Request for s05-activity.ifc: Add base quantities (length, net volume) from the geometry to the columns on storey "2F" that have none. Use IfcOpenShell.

First a look at what the model holds.

```python
import ifcopenshell
import ifcopenshell.util.element
import ifcopenshell.util.unit

model = ifcopenshell.open("s05-activity.ifc")
print(model.schema)
for unit_type in ("LENGTHUNIT", "AREAUNIT", "VOLUMEUNIT"):
    print(unit_type, ifcopenshell.util.unit.calculate_unit_scale(model, unit_type))
storey = next(s for s in model.by_type("IfcBuildingStorey") if s.Name == "2F")
columns = [e for e in ifcopenshell.util.element.get_decomposition(storey) if e.is_a("IfcColumn")]
for e in sorted(columns, key=lambda e: e.id()):
    print(e.id(), e.is_a(), e.Name, list(ifcopenshell.util.element.get_psets(e, qtos_only=True)), sep=" | ")
```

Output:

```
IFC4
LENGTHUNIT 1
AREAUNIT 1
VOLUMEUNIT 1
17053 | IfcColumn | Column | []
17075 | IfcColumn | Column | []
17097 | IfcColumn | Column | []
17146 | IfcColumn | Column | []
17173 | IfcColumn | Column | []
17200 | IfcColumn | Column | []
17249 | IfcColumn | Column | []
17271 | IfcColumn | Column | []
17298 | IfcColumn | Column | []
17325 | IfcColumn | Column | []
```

```python
import ifcopenshell
import ifcopenshell.api.pset
import ifcopenshell.geom
import ifcopenshell.util.element
import ifcopenshell.util.shape
import ifcopenshell.util.unit

model = ifcopenshell.open("s05-activity.ifc")
unit_scale = ifcopenshell.util.unit.calculate_unit_scale(model)
volume_scale = ifcopenshell.util.unit.calculate_unit_scale(model, "VOLUMEUNIT")
settings = ifcopenshell.geom.settings()

storey = next(s for s in model.by_type("IfcBuildingStorey") if s.Name == "2F")
columns = [e for e in ifcopenshell.util.element.get_decomposition(storey) if e.is_a("IfcColumn")]

for e in sorted(columns, key=lambda e: e.id()):
    if ifcopenshell.util.element.get_psets(e, qtos_only=True, should_inherit=False):
        continue
    # Geometry comes back in metres, in the element's own axes.
    shape = ifcopenshell.geom.create_shape(settings, e)
    values = {
        "Length": ifcopenshell.util.shape.get_z(shape.geometry) / unit_scale,
        "NetVolume": ifcopenshell.util.shape.get_volume(shape.geometry) / volume_scale,
    }
    qto = ifcopenshell.api.pset.add_qto(model, product=e, name="Qto_ColumnBaseQuantities")
    ifcopenshell.api.pset.edit_qto(model, qto=qto, properties=values)
    print(e.id(), {k: round(v, 3) for k, v in values.items()})

model.write("s05-activity-out.ifc")
```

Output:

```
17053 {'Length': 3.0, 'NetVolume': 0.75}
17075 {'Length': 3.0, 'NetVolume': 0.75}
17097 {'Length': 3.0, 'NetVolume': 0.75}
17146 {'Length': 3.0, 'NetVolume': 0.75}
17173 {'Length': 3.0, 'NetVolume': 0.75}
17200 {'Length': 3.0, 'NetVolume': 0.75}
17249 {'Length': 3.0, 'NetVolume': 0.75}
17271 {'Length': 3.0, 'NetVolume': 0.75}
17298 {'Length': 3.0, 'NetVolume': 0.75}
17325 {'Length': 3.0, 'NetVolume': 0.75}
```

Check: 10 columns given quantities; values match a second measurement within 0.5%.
